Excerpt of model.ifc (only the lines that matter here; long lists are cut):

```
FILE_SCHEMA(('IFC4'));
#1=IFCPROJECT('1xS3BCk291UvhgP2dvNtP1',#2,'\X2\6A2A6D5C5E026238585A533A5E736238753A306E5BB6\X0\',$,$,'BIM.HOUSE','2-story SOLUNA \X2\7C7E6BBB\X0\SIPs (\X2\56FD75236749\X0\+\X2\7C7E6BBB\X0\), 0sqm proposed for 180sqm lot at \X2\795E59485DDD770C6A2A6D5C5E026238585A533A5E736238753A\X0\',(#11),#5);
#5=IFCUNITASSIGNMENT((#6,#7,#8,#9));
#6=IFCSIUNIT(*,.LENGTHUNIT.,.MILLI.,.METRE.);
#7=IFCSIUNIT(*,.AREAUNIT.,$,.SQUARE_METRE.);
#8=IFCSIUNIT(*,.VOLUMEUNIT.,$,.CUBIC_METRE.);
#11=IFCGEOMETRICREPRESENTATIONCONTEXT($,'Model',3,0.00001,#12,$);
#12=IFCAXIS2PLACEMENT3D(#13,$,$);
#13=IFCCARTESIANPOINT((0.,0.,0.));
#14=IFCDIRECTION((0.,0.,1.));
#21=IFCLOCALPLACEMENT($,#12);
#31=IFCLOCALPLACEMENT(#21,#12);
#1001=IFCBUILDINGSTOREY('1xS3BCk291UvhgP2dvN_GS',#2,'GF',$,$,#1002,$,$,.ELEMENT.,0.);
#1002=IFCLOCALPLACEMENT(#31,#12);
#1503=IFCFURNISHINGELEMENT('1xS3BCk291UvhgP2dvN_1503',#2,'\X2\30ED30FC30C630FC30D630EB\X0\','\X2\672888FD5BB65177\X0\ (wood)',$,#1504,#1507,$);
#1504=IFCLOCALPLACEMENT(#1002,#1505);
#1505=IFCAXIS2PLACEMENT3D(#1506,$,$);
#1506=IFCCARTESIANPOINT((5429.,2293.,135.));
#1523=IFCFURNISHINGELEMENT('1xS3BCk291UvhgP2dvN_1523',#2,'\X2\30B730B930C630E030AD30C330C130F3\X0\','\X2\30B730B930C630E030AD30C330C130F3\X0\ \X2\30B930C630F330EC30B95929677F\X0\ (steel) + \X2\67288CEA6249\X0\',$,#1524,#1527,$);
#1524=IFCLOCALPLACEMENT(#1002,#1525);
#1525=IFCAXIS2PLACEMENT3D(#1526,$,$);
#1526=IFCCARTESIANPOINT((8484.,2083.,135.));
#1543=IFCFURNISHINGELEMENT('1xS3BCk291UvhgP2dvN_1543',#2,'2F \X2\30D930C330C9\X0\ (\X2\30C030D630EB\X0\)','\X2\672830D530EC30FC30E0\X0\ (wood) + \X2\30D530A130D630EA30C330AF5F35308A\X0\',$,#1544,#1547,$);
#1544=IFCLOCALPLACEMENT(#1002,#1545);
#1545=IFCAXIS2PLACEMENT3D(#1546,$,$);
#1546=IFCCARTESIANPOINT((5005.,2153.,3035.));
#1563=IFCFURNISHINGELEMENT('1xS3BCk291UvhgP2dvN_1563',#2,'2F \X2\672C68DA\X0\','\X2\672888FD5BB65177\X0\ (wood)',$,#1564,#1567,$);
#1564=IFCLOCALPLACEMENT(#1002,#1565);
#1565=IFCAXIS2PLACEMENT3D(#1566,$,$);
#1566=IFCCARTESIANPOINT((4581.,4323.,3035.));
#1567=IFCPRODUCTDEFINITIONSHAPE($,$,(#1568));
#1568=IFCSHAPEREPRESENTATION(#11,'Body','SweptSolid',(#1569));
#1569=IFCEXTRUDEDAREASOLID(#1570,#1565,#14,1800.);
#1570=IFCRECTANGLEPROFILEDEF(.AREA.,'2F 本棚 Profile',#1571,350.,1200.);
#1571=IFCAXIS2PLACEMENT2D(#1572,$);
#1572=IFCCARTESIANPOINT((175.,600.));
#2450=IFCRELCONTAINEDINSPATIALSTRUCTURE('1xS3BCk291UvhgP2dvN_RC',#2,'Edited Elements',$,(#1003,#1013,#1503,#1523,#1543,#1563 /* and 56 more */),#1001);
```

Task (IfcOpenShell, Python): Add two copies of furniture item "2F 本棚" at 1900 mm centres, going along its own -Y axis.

```python
import ifcopenshell
import ifcopenshell.api.geometry
import ifcopenshell.api.root
import ifcopenshell.util.element
import ifcopenshell.util.placement
import ifcopenshell.util.unit

model = ifcopenshell.open("model.ifc")
unit_scale = ifcopenshell.util.unit.calculate_unit_scale(model)


def reuse_history(source, copy):
    """copy_class also copies each property set's owner history, people and application; keep the originals."""
    for rel in copy.IsDefinedBy:
        if rel.is_a("IfcRelDefinesByProperties") and (history := rel.RelatingPropertyDefinition.OwnerHistory):
            rel.RelatingPropertyDefinition.OwnerHistory = source.OwnerHistory
            ifcopenshell.util.element.remove_deep2(model, history)


source = model.by_guid("1xS3BCk291UvhgP2dvN_1563")
base = ifcopenshell.util.placement.get_local_placement(source.ObjectPlacement)
step = -base[:3, 1] * 1.9 / unit_scale

for i in range(1, 3):
    copy = ifcopenshell.api.root.copy_class(model, product=source)
    copy.Representation = ifcopenshell.util.element.copy_deep(
        model, source.Representation, exclude=["IfcGeometricRepresentationContext", "IfcRepresentationMap"]
    )
    reuse_history(source, copy)
    matrix = base.copy()
    matrix[:3, 3] += i * step
    print("added at", matrix[:3, 3].round(3) + 0.0)
    ifcopenshell.api.geometry.edit_object_placement(model, product=copy, matrix=matrix, is_si=False)

model.write("model_updated.ifc")
```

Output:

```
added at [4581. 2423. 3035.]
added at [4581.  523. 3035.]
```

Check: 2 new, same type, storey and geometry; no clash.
